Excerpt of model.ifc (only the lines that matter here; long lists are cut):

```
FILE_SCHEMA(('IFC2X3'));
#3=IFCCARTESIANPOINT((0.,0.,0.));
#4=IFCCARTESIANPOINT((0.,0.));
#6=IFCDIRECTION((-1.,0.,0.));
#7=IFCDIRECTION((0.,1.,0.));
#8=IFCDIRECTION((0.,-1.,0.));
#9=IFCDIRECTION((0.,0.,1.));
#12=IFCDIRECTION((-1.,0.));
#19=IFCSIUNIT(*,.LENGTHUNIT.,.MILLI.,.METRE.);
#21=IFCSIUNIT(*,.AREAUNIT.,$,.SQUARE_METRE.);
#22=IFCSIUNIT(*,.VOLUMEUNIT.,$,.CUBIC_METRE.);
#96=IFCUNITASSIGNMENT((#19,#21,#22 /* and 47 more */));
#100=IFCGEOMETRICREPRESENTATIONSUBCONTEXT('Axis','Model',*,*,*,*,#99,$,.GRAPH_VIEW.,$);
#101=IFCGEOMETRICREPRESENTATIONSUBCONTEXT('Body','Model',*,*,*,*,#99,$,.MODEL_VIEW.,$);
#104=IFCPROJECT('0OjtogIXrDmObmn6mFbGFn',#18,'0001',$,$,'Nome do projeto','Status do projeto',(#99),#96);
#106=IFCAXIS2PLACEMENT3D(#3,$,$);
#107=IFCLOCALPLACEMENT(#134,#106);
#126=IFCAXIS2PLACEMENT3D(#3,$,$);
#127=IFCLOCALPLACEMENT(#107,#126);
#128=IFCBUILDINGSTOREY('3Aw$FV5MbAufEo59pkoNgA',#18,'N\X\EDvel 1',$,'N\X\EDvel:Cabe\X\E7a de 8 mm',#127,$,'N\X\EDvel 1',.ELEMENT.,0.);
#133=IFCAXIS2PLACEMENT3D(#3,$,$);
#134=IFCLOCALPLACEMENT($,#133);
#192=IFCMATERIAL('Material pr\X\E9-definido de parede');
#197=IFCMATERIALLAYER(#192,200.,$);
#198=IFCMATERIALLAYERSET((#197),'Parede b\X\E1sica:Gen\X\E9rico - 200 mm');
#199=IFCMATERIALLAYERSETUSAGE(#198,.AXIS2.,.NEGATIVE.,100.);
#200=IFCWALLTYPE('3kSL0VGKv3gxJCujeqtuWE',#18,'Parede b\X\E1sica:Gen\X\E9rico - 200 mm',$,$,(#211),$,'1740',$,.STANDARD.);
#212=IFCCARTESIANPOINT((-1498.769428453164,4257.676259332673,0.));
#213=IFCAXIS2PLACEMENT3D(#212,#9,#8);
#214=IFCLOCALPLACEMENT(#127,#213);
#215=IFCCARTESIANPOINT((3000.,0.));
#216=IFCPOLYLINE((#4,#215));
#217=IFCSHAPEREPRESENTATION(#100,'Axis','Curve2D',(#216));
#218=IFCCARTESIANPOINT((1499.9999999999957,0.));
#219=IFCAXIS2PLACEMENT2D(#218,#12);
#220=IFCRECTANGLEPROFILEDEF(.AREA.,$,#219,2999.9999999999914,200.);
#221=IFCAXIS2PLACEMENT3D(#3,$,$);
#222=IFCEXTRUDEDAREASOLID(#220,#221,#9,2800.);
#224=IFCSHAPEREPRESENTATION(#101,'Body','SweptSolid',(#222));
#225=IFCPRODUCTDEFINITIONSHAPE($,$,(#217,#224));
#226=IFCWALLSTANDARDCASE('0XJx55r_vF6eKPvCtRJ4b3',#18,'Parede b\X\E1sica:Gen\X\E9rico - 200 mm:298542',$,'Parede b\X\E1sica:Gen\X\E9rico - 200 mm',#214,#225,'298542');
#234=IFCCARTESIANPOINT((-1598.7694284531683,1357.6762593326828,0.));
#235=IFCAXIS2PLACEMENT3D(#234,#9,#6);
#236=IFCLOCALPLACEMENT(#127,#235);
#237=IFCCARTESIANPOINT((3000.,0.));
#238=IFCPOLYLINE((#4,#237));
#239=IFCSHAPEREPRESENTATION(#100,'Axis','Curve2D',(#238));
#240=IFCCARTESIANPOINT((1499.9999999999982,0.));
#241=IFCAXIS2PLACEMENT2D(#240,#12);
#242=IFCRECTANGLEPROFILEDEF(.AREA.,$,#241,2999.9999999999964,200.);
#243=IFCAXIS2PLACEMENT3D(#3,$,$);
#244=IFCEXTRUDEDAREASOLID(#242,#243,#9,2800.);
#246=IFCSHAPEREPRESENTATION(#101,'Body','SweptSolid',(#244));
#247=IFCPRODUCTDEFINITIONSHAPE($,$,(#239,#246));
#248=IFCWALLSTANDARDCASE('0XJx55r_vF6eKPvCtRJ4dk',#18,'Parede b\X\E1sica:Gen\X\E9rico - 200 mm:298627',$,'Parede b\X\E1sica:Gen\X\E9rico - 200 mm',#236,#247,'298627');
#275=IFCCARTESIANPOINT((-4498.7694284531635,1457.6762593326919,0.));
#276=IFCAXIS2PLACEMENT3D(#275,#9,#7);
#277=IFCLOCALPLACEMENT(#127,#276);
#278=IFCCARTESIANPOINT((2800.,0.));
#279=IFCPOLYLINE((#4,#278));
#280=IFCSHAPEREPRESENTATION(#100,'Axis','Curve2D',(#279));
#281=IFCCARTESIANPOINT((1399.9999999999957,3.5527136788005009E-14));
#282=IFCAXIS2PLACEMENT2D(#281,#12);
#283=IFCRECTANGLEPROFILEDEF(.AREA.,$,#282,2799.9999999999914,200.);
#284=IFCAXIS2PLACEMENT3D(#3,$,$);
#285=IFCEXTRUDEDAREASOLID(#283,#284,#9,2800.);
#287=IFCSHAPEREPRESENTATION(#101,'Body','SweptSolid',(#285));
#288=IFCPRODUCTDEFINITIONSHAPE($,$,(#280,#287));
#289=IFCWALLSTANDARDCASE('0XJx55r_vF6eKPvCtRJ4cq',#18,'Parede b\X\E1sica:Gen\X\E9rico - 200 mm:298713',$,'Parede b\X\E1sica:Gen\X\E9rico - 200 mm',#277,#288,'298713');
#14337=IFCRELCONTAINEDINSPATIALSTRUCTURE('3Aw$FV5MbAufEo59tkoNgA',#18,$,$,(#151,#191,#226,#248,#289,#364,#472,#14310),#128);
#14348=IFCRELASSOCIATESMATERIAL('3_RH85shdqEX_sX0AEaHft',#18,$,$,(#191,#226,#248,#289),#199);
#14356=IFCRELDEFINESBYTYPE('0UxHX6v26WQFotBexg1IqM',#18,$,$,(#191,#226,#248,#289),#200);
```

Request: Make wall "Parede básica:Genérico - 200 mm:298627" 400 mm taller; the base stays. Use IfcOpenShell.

```python
import ifcopenshell
import ifcopenshell.geom
import ifcopenshell.util.representation
import ifcopenshell.util.shape

model = ifcopenshell.open("model.ifc")
settings = ifcopenshell.geom.settings()


def volume(element):
    """Net volume in cubic metres, openings subtracted."""
    shape = ifcopenshell.geom.create_shape(settings, element)
    return ifcopenshell.util.shape.get_volume(shape.geometry)


wall = model.by_guid("0XJx55r_vF6eKPvCtRJ4dk")
before = volume(wall)

body = ifcopenshell.util.representation.get_representation(wall, "Model", "Body")
solid = body.Items[0]
old_height = solid.Depth
solid.Depth += 400.0
after = volume(wall)

print(f"height {old_height:g} -> {solid.Depth:g}, volume {before:.3f} -> {after:.3f} m3")

model.write("model_edited.ifc")
```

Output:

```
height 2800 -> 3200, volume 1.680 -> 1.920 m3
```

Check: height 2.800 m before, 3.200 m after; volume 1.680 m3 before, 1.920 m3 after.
